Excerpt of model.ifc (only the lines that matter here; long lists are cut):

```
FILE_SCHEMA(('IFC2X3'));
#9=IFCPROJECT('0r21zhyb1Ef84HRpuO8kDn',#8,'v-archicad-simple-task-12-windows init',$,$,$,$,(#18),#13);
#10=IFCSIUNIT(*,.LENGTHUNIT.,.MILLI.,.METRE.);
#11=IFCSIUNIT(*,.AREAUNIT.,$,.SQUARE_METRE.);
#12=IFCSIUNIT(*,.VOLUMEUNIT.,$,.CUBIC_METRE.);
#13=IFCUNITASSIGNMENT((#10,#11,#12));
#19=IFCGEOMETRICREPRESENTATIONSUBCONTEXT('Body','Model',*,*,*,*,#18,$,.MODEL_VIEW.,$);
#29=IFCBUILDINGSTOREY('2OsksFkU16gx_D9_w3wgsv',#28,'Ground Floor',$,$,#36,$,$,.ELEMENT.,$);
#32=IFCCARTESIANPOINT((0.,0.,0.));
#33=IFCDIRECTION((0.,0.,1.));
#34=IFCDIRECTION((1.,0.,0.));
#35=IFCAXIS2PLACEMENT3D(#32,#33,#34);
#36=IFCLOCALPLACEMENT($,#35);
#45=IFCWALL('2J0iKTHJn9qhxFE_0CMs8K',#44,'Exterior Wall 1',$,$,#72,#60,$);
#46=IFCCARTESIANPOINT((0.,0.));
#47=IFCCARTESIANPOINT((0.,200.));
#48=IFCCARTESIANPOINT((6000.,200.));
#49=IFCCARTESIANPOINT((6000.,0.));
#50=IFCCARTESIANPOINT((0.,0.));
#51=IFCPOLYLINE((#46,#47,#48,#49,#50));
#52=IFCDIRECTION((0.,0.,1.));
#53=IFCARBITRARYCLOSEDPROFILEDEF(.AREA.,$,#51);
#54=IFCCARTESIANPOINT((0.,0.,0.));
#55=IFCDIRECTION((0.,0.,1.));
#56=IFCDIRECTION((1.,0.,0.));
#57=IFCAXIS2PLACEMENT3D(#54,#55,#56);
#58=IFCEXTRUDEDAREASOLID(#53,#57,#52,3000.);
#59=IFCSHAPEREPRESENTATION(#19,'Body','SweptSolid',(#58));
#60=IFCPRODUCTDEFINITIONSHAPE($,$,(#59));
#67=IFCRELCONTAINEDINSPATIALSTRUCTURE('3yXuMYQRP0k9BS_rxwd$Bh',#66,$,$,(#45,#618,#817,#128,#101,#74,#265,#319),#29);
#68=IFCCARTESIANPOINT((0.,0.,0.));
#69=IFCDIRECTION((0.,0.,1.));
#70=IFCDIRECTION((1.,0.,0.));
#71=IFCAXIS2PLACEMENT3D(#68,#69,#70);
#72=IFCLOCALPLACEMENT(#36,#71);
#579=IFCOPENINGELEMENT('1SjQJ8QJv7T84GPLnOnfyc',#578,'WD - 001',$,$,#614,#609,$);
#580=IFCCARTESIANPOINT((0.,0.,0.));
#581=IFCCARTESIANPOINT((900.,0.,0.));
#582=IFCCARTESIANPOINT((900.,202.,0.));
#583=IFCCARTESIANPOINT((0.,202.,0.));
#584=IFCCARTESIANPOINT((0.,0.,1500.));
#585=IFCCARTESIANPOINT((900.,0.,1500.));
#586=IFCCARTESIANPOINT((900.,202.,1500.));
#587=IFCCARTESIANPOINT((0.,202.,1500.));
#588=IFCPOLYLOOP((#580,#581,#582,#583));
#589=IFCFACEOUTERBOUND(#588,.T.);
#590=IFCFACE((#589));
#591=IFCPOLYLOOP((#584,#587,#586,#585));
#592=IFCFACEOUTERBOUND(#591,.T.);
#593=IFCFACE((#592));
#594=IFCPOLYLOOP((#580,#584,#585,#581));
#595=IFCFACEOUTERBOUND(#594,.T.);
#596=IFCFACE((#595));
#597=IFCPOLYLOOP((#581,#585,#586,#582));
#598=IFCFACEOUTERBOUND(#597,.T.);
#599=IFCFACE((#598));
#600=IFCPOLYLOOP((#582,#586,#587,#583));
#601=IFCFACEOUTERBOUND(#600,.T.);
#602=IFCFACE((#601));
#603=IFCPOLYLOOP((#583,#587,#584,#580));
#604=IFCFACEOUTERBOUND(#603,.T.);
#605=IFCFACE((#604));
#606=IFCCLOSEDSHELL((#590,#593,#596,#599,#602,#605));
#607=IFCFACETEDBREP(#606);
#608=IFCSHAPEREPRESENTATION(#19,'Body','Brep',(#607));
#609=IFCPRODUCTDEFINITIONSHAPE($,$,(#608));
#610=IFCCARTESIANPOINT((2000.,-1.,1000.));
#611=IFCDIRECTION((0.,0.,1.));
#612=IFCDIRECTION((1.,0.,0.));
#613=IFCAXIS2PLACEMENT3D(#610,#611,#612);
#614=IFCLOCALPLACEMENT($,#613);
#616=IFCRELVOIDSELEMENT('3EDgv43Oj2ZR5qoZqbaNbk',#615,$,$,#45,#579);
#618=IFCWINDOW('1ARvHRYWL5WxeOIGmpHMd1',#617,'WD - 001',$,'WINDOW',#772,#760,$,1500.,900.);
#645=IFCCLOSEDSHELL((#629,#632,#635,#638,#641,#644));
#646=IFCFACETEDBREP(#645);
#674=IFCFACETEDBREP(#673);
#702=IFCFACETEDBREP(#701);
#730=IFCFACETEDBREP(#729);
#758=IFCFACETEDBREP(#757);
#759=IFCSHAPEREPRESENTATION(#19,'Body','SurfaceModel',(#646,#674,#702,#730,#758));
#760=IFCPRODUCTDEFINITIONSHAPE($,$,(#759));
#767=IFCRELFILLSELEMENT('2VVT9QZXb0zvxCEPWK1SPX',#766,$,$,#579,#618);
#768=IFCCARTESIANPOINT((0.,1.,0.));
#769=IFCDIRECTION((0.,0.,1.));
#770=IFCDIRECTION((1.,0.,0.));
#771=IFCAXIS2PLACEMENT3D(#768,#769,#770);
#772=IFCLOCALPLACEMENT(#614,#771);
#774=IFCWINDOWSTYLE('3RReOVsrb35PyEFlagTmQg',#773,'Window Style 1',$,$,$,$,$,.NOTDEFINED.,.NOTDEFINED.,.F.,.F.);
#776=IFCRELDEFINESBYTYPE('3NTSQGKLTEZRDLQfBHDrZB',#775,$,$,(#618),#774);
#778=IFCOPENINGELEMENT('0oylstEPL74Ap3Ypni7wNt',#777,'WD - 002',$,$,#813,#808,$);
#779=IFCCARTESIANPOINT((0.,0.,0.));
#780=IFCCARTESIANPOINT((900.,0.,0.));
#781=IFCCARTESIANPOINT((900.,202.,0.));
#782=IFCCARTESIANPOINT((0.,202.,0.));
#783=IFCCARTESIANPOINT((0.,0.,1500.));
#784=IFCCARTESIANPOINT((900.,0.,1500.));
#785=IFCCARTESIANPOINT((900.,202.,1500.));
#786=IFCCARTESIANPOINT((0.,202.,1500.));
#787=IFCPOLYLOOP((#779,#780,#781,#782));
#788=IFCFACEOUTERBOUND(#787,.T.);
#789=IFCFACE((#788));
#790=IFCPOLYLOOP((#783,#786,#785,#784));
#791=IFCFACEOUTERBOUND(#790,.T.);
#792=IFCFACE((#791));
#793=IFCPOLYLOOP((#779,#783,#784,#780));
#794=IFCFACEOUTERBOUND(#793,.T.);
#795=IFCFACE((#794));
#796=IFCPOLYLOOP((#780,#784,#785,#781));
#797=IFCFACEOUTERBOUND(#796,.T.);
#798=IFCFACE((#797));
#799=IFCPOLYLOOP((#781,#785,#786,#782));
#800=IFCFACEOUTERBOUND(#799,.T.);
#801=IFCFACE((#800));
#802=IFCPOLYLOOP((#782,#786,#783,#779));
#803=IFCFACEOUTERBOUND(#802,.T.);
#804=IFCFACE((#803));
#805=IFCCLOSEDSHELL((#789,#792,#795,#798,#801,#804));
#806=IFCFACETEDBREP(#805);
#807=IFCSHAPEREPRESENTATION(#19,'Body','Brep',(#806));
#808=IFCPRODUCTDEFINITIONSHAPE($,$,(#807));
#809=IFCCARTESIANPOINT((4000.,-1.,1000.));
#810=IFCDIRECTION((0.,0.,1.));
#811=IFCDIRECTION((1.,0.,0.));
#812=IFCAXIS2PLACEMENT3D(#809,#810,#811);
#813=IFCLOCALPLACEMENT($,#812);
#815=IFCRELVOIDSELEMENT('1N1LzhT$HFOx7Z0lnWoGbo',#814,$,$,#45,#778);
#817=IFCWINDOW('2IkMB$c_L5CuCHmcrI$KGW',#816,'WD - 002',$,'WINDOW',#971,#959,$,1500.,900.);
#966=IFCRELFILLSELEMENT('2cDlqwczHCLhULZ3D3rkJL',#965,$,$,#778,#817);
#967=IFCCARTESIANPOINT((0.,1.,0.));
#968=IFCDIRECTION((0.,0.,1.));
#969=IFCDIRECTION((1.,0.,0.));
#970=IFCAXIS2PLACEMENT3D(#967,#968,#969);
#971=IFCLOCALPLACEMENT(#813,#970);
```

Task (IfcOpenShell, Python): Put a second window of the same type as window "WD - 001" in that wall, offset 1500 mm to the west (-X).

```python
import ifcopenshell
import ifcopenshell.api.feature
import ifcopenshell.api.geometry
import ifcopenshell.api.root
import ifcopenshell.geom
import ifcopenshell.util.element
import ifcopenshell.util.placement
import ifcopenshell.util.shape
import ifcopenshell.util.unit

model = ifcopenshell.open("model.ifc")
unit_scale = ifcopenshell.util.unit.calculate_unit_scale(model)
settings = ifcopenshell.geom.settings()


def volume(element):
    """Net volume in cubic metres, openings subtracted."""
    shape = ifcopenshell.geom.create_shape(settings, element)
    return ifcopenshell.util.shape.get_volume(shape.geometry)


window = model.by_guid("1ARvHRYWL5WxeOIGmpHMd1")
opening = window.FillsVoids[0].RelatingOpeningElement
wall = opening.VoidsElements[0].RelatingBuildingElement
before = volume(wall)
shift = ifcopenshell.util.placement.get_local_placement(wall.ObjectPlacement)[:3, 0] * -1.5 / unit_scale

# copy_class copies the void relationship, type, container and properties, but no geometry.
new_opening = ifcopenshell.api.root.copy_class(model, product=opening)
new_opening.Representation = ifcopenshell.util.element.copy_deep(
    model, opening.Representation, exclude=["IfcGeometricRepresentationContext", "IfcRepresentationMap"]
)
new_window = ifcopenshell.api.root.copy_class(model, product=window)
new_window.Representation = ifcopenshell.util.element.copy_deep(
    model, window.Representation, exclude=["IfcGeometricRepresentationContext", "IfcRepresentationMap"]
)
fills = ifcopenshell.api.feature.add_filling(model, opening=new_opening, element=new_window)
fills.OwnerHistory = new_window.OwnerHistory  # required in IFC2X3

for old, new in ((opening, new_opening), (window, new_window)):
    matrix = ifcopenshell.util.placement.get_local_placement(old.ObjectPlacement)
    matrix[:3, 3] += shift
    ifcopenshell.api.geometry.edit_object_placement(model, product=new, matrix=matrix, is_si=False)

after = volume(wall)

print(f"wall volume {before:.3f} -> {after:.3f} m3")

model.write("model_updated.ifc")
```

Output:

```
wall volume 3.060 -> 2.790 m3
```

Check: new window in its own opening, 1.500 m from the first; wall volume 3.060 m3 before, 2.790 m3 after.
